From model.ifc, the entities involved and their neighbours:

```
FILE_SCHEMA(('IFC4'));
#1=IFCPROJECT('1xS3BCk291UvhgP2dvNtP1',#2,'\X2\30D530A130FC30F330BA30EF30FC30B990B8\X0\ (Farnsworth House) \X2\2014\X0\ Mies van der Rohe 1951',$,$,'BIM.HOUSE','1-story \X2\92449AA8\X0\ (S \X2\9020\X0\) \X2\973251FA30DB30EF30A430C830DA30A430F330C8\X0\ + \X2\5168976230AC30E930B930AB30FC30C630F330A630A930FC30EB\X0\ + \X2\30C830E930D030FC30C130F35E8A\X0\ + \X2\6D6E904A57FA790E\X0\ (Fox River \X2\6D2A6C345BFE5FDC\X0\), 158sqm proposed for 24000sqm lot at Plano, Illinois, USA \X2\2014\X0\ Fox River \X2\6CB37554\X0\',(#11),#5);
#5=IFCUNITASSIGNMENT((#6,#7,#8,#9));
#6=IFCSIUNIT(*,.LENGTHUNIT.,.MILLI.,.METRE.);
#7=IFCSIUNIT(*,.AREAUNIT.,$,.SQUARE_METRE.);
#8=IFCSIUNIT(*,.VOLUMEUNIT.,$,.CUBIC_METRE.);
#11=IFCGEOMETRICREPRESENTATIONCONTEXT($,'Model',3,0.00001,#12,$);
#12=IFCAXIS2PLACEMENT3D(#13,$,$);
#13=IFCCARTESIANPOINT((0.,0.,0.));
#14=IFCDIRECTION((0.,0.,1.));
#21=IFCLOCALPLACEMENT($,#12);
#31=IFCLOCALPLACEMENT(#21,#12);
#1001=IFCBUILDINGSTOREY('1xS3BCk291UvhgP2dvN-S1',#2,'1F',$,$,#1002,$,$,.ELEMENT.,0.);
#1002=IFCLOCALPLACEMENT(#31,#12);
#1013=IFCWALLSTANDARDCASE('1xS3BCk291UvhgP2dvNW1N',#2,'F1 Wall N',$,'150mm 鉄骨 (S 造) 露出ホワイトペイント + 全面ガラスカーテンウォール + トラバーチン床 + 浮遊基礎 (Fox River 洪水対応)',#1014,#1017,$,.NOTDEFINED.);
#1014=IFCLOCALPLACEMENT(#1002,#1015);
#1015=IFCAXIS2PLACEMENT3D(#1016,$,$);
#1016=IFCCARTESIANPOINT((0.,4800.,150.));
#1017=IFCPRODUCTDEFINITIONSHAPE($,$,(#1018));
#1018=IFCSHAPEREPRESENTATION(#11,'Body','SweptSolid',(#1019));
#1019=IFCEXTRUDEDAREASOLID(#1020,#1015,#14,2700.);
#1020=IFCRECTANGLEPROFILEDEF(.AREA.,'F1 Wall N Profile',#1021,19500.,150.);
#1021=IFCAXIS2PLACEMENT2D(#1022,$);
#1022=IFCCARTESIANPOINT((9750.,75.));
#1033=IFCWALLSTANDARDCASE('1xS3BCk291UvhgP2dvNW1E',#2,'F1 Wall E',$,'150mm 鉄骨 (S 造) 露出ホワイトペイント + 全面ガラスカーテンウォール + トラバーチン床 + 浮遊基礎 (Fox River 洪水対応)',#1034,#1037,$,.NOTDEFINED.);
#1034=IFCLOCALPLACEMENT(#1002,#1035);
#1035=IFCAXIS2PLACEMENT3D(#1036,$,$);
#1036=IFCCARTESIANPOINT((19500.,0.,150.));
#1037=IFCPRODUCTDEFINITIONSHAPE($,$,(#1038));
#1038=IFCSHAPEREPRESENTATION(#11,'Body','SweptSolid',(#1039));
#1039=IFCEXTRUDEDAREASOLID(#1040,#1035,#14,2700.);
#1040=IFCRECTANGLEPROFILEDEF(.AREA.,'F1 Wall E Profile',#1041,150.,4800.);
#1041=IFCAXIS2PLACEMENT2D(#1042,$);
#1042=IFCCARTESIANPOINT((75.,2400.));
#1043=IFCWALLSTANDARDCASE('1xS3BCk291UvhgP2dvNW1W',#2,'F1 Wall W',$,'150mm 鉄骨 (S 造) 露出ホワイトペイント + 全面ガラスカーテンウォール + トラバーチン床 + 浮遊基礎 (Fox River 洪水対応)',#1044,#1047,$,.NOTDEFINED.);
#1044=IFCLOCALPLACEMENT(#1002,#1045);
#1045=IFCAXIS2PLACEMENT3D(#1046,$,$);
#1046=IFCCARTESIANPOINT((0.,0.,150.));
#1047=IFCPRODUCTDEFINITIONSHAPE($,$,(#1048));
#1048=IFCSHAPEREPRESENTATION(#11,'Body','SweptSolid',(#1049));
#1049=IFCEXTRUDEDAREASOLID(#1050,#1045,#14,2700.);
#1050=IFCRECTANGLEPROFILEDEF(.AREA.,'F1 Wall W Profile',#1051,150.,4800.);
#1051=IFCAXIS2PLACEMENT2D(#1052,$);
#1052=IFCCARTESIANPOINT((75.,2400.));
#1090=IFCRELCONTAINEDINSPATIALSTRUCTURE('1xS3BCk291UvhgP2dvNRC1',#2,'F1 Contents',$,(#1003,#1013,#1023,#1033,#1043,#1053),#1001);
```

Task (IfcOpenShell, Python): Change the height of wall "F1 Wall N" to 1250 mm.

```python
import ifcopenshell
import ifcopenshell.geom
import ifcopenshell.util.shape
import ifcopenshell.util.unit

model = ifcopenshell.open("model.ifc")
unit_scale = ifcopenshell.util.unit.calculate_unit_scale(model)
settings = ifcopenshell.geom.settings()


def volume(element):
    """Net volume in cubic metres, openings subtracted."""
    shape = ifcopenshell.geom.create_shape(settings, element)
    return ifcopenshell.util.shape.get_volume(shape.geometry)


wall = model.by_id(1013)
before = volume(wall)

body = next(r for r in wall.Representation.Representations if r.RepresentationIdentifier == "Body")
solid = body.Items[0]
old_height = solid.Depth
solid.Depth = 1.25 / unit_scale
after = volume(wall)

print(f"height {old_height:g} -> {solid.Depth:g}, volume {before:.3f} -> {after:.3f} m3")

model.write("model-out.ifc")
```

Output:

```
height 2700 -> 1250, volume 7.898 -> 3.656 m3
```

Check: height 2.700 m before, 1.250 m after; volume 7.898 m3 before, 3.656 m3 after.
